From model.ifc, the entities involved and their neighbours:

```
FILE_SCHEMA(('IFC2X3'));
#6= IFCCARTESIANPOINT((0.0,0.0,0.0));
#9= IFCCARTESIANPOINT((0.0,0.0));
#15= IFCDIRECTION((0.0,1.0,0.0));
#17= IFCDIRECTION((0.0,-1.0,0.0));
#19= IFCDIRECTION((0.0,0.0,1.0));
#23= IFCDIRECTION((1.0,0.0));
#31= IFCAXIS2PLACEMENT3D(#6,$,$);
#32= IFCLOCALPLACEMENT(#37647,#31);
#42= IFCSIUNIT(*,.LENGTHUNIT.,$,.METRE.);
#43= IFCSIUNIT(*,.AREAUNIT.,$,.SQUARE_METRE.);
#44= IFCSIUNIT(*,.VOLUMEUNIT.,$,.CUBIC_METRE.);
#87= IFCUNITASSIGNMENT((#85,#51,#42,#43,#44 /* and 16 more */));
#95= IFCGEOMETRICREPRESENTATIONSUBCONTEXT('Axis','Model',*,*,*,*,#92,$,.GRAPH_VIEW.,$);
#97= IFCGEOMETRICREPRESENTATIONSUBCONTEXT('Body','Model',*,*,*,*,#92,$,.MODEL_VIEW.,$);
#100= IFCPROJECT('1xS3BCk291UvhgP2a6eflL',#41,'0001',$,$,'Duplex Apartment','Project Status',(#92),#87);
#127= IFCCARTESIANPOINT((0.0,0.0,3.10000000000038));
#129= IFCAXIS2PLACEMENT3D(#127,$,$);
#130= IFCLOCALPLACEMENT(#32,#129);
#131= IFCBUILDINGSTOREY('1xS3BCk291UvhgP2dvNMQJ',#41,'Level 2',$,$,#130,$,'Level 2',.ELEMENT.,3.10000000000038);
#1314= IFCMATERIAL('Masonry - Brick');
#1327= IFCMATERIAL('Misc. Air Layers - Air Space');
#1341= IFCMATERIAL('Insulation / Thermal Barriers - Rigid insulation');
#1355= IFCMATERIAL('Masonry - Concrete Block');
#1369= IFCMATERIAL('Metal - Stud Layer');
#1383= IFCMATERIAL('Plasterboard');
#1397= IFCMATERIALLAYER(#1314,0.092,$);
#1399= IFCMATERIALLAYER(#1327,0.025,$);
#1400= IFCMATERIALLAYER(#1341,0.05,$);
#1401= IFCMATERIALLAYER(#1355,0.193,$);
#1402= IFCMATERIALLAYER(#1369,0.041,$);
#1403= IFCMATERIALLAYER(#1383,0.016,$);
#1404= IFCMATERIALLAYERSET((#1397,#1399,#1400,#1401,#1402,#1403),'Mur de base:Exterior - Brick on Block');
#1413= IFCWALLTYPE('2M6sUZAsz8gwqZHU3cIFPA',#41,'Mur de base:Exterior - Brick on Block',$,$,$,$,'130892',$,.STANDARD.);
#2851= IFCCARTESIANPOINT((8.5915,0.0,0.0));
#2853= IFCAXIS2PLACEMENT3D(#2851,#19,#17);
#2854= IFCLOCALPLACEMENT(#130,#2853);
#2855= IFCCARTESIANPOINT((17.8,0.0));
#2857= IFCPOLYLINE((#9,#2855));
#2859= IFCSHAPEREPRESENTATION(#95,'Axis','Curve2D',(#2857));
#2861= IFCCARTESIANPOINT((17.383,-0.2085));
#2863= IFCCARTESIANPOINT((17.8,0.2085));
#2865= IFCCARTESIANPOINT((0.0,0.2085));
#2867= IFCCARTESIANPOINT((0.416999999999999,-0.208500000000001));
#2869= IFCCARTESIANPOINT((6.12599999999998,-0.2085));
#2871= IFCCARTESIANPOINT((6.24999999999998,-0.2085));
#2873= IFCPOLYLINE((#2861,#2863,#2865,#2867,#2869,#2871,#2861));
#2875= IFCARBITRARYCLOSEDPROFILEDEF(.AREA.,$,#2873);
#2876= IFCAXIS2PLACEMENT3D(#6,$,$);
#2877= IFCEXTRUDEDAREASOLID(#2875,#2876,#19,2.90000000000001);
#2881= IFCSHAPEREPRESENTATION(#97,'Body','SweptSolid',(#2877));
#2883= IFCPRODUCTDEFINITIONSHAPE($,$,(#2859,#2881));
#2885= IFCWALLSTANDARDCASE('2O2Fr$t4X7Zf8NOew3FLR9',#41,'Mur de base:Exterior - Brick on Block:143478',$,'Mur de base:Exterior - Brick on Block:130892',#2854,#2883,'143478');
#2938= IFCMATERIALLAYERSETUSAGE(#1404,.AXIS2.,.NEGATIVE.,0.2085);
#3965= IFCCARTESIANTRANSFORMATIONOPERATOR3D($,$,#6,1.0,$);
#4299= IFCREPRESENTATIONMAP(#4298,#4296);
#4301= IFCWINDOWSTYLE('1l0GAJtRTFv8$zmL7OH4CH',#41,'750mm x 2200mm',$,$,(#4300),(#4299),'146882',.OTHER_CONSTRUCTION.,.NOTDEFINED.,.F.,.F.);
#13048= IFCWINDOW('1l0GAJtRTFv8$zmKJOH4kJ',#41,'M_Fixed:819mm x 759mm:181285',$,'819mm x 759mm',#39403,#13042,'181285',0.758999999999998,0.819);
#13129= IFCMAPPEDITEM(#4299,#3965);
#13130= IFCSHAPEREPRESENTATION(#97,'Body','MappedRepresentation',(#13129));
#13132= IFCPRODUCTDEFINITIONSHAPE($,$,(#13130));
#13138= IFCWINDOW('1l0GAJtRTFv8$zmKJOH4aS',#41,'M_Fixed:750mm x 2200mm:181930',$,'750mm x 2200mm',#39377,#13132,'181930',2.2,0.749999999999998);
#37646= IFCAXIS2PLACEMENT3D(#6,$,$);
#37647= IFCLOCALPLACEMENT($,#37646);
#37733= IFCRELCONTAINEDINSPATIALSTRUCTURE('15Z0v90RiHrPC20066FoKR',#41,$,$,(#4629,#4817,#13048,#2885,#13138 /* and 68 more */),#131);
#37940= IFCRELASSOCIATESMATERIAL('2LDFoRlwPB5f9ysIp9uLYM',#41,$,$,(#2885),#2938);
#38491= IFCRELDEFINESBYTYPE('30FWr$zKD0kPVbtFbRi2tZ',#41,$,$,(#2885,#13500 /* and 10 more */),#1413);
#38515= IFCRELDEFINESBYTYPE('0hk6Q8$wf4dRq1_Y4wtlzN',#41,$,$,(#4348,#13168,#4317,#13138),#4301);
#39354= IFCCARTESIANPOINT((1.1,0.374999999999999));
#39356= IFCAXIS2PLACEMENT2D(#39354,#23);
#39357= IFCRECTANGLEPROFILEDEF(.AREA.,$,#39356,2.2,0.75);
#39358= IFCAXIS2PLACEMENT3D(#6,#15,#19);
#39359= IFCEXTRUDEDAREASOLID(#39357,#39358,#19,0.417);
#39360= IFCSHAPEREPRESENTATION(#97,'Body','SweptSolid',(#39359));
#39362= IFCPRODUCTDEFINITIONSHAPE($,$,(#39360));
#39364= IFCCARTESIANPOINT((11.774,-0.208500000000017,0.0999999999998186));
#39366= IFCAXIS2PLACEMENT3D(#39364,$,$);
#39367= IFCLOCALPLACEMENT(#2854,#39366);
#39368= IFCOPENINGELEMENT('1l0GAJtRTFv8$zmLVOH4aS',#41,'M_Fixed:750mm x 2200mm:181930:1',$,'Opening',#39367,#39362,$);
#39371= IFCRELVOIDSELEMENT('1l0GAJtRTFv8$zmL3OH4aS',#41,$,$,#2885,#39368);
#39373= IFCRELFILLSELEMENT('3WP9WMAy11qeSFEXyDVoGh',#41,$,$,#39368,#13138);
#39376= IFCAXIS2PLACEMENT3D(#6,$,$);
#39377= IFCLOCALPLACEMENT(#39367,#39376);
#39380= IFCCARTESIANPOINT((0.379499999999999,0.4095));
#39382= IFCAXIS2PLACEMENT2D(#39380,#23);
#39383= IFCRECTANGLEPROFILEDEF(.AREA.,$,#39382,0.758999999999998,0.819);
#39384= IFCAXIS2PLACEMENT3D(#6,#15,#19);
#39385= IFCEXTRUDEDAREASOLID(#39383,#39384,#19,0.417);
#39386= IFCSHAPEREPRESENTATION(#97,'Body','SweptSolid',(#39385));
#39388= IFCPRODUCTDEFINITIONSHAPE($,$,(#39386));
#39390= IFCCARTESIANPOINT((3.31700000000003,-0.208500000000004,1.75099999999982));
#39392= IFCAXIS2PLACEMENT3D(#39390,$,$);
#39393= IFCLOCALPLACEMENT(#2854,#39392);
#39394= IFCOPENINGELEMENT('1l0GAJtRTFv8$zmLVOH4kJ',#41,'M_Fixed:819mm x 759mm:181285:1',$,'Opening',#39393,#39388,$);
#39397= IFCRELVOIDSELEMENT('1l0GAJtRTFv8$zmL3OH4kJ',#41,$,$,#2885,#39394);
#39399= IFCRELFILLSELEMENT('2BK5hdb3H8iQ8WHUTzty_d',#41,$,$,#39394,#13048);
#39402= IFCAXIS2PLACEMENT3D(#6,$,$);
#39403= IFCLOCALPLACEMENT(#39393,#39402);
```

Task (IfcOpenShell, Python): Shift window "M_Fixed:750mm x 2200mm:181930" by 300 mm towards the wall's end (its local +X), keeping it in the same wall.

```python
import ifcopenshell
import ifcopenshell.api.geometry
import ifcopenshell.util.placement

model = ifcopenshell.open("model.ifc")

window = model.by_id(13138)
opening = window.FillsVoids[0].RelatingOpeningElement
wall = opening.VoidsElements[0].RelatingBuildingElement

wall_matrix = ifcopenshell.util.placement.get_local_placement(wall.ObjectPlacement)
shift = wall_matrix[:3, 0] * 0.3
before = ifcopenshell.util.placement.get_local_placement(window.ObjectPlacement)[:3, 3].copy()

# The window is placed relative to its opening, so it follows when the opening moves.
matrix = ifcopenshell.util.placement.get_local_placement(opening.ObjectPlacement)
matrix[:3, 3] += shift
ifcopenshell.api.geometry.edit_object_placement(
    model, product=opening, matrix=matrix, is_si=False, should_transform_children=True
)

after = ifcopenshell.util.placement.get_local_placement(window.ObjectPlacement)[:3, 3]
print("window moved by", (after - before).round(3) + 0.0)

model.write("model_edited.ifc")
```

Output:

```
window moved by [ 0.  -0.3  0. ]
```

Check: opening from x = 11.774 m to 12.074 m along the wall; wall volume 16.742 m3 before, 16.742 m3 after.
